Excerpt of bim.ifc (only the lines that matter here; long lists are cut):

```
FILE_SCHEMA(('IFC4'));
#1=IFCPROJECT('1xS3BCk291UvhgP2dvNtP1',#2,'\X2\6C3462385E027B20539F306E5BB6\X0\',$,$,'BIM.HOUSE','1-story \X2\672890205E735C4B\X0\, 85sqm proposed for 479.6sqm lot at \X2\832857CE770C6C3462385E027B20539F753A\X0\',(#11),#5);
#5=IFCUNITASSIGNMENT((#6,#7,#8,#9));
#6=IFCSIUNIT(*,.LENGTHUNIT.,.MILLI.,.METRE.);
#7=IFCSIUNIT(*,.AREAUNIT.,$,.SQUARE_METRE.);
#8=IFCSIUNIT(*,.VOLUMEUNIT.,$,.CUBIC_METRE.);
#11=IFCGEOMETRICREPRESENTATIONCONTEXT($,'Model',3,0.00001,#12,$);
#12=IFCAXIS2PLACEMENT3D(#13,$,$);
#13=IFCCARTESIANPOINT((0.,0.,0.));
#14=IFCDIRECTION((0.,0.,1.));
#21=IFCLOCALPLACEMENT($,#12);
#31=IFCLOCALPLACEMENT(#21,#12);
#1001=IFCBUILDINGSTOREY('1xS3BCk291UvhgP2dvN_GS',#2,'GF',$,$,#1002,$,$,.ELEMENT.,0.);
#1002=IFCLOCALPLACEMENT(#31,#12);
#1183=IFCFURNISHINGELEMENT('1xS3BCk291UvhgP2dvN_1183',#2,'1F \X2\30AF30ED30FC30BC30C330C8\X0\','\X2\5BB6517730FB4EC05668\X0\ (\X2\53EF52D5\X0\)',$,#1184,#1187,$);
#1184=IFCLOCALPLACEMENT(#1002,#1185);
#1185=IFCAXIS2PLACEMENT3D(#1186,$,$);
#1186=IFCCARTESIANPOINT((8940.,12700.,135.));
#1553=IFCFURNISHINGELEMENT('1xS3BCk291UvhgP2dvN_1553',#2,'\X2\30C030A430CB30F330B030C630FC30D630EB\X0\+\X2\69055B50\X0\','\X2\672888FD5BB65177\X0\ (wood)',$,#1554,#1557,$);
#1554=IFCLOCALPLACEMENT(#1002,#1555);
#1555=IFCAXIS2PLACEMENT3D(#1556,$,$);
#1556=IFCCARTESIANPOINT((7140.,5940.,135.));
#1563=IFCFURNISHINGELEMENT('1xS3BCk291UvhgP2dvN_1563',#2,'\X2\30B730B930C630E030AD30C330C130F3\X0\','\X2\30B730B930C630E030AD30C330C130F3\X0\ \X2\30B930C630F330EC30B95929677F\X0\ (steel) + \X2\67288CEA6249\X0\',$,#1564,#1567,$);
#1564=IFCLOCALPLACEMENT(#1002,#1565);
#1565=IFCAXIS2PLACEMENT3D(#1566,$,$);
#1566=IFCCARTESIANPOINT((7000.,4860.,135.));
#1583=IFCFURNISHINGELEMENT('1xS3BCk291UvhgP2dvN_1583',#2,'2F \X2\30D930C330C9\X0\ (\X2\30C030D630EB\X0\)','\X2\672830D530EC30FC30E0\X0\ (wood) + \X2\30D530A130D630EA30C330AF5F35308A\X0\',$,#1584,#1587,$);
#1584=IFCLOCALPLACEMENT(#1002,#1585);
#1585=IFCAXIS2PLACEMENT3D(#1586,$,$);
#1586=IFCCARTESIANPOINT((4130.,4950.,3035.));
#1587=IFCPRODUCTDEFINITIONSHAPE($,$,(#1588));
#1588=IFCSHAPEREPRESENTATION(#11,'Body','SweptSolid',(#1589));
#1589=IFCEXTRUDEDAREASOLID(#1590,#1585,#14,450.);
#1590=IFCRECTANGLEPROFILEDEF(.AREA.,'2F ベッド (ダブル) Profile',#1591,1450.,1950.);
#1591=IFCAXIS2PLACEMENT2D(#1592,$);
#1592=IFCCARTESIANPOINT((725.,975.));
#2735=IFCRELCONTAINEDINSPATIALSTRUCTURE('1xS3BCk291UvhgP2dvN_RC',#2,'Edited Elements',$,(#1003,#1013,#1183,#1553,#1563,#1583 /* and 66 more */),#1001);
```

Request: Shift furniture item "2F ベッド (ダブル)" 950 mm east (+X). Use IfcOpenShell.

```python
import ifcopenshell
import ifcopenshell.api.geometry
import ifcopenshell.util.placement
import ifcopenshell.util.unit

model = ifcopenshell.open("bim.ifc")
unit_scale = ifcopenshell.util.unit.calculate_unit_scale(model)

item = model.by_guid("1xS3BCk291UvhgP2dvN_1583")
matrix = ifcopenshell.util.placement.get_local_placement(item.ObjectPlacement)
matrix[0, 3] += 0.95 / unit_scale
ifcopenshell.api.geometry.edit_object_placement(model, product=item, matrix=matrix, is_si=False)

print(ifcopenshell.util.placement.get_local_placement(item.ObjectPlacement).round(3) + 0.0)

model.write("bim_edited.ifc")
```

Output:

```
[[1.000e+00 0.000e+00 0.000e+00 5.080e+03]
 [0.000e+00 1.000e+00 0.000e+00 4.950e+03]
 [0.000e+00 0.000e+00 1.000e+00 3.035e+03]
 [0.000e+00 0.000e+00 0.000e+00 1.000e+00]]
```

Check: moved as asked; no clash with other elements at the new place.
